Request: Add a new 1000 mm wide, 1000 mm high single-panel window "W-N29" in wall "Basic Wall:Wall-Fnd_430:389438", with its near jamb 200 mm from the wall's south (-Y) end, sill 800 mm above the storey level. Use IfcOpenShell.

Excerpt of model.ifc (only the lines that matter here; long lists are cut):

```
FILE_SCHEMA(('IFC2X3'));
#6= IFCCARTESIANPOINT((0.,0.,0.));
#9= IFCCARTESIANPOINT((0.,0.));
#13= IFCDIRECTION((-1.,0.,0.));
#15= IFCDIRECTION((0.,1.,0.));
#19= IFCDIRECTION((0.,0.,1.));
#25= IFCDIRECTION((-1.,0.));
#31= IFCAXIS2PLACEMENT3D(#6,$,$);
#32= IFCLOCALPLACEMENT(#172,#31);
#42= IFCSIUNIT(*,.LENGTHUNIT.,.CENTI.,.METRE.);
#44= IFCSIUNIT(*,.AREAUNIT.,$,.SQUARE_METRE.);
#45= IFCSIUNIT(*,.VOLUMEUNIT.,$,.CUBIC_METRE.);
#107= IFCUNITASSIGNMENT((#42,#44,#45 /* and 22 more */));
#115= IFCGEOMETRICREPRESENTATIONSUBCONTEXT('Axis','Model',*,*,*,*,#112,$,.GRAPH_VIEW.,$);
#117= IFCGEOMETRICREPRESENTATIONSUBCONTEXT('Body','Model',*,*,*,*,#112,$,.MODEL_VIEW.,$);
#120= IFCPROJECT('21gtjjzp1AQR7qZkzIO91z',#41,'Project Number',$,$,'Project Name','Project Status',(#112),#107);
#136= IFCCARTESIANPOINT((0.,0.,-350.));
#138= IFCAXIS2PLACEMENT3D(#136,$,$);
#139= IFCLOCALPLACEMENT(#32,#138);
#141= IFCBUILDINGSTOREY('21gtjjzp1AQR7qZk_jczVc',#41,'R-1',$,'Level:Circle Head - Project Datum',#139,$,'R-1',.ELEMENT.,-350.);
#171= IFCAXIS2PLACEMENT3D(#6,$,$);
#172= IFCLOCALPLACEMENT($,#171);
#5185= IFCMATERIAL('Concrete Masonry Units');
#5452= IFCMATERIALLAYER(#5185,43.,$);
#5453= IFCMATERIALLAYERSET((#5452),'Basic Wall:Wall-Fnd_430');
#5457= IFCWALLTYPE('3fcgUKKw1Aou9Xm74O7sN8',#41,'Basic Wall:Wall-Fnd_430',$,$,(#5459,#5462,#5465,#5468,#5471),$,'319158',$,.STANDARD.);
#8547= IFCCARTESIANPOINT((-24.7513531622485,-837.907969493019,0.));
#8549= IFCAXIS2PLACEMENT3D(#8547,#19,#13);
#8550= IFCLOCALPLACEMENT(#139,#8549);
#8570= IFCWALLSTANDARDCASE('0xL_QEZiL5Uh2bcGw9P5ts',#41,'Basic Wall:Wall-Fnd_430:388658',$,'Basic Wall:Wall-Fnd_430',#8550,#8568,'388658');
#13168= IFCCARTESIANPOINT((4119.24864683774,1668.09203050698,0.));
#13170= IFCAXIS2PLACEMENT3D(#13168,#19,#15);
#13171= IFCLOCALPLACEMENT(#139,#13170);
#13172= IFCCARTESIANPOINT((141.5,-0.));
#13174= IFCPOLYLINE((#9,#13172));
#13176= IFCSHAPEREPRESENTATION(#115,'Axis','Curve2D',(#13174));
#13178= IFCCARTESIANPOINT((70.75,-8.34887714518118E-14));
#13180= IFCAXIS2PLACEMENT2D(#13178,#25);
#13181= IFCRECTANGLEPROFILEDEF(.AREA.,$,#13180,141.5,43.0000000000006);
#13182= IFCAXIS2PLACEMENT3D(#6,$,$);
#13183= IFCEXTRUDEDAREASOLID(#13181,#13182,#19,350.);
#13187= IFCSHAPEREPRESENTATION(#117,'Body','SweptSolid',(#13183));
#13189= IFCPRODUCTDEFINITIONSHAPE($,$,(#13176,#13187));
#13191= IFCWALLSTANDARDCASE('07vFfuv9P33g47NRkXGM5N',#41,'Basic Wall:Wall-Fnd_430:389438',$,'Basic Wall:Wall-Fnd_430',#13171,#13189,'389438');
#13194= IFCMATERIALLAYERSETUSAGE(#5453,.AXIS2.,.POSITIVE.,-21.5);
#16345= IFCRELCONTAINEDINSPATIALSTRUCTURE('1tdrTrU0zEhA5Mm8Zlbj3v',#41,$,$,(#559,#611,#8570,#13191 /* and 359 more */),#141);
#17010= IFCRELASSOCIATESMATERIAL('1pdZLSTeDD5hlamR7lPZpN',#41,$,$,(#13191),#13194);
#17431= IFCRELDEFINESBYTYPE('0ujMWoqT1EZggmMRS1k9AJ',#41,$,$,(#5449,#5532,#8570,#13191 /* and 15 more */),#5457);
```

```python
import numpy as np
import ifcopenshell
import ifcopenshell.api.feature
import ifcopenshell.api.geometry
import ifcopenshell.api.root
import ifcopenshell.api.spatial
import ifcopenshell.api.type
import ifcopenshell.geom
import ifcopenshell.util.element
import ifcopenshell.util.placement
import ifcopenshell.util.representation
import ifcopenshell.util.shape
import ifcopenshell.util.unit

model = ifcopenshell.open("model.ifc")
unit_scale = ifcopenshell.util.unit.calculate_unit_scale(model)
settings = ifcopenshell.geom.settings()


def volume(element):
    """Net volume in cubic metres, openings subtracted."""
    shape = ifcopenshell.geom.create_shape(settings, element)
    return ifcopenshell.util.shape.get_volume(shape.geometry)


wall = model.by_guid("07vFfuv9P33g47NRkXGM5N")
storey = ifcopenshell.util.element.get_container(wall, ifc_class="IfcBuildingStorey")
context = ifcopenshell.util.representation.get_context(model, "Model", "Body", "MODEL_VIEW")
before = volume(wall)

width, height, from_end, sill = 1, 1, 0.2, 0.8  # metres

# The wall runs along its own X axis, and the end named is its -X end.
wall_shape = ifcopenshell.geom.create_shape(settings, wall)
x, y, z = ifcopenshell.util.shape.get_vertices(wall_shape.geometry).T
start = x.min() + from_end
face, thickness = float(y.min()), float(y.max() - y.min())
wall_matrix = ifcopenshell.util.placement.get_local_placement(wall.ObjectPlacement)
level = ifcopenshell.util.placement.get_local_placement(storey.ObjectPlacement)[2, 3]


def in_wall(x, y):
    """Placement at x, y metres in the wall's axes, at sill height."""
    matrix = wall_matrix.copy()
    matrix[:, 3] = wall_matrix @ np.array([x / unit_scale, y / unit_scale, 0.0, 1.0])
    matrix[2, 3] = level + sill / unit_scale
    return matrix


# Opening: a box that overshoots both wall faces by 50 mm.
opening = ifcopenshell.api.root.create_entity(model, ifc_class="IfcOpeningElement")
box = ifcopenshell.api.geometry.add_wall_representation(
    model, context=context, length=width, height=height, thickness=thickness + 0.1
)
ifcopenshell.api.geometry.assign_representation(model, product=opening, representation=box)
ifcopenshell.api.geometry.edit_object_placement(model, product=opening, matrix=in_wall(start, face - 0.05), is_si=False)
ifcopenshell.api.feature.add_feature(model, feature=opening, element=wall)

window = ifcopenshell.api.root.create_entity(model, ifc_class="IfcWindow", name="W-N29")
window.OverallWidth, window.OverallHeight = width / unit_scale, height / unit_scale
body = ifcopenshell.api.geometry.add_window_representation(
    model,
    context=context,
    overall_width=window.OverallWidth,
    overall_height=window.OverallHeight,
    partition_type="SINGLE_PANEL",
)
ifcopenshell.api.geometry.assign_representation(model, product=window, representation=body)
ifcopenshell.api.spatial.assign_container(model, products=[window], relating_structure=storey)
fills = ifcopenshell.api.feature.add_filling(model, opening=opening, element=window)
fills.OwnerHistory = window.OwnerHistory  # required in IFC2X3

# IFC2X3 keeps the operation on the window style.
style = ifcopenshell.api.root.create_entity(model, ifc_class="IfcWindowStyle", name="W-N29")
style.OperationType, style.ConstructionType = "SINGLE_PANEL", "NOTDEFINED"
style.ParameterTakesPrecedence = style.Sizeable = False
ifcopenshell.api.type.assign_type(model, related_objects=[window], relating_type=style)

# Centre the window in the wall's thickness.
ifcopenshell.api.geometry.edit_object_placement(model, product=window, matrix=in_wall(start, face), is_si=False)
window_shape = ifcopenshell.geom.create_shape(settings, window)
depth = ifcopenshell.util.shape.get_vertices(window_shape.geometry)[:, 1]
offset = face + thickness / 2 - (depth.min() + depth.max()) / 2
ifcopenshell.api.geometry.edit_object_placement(model, product=window, matrix=in_wall(start, offset), is_si=False)

after = volume(wall)

print(f"wall volume {before:.3f} -> {after:.3f} m3")

model.write("model_rev.ifc")
```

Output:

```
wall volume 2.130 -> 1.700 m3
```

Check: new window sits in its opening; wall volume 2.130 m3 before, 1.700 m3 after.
